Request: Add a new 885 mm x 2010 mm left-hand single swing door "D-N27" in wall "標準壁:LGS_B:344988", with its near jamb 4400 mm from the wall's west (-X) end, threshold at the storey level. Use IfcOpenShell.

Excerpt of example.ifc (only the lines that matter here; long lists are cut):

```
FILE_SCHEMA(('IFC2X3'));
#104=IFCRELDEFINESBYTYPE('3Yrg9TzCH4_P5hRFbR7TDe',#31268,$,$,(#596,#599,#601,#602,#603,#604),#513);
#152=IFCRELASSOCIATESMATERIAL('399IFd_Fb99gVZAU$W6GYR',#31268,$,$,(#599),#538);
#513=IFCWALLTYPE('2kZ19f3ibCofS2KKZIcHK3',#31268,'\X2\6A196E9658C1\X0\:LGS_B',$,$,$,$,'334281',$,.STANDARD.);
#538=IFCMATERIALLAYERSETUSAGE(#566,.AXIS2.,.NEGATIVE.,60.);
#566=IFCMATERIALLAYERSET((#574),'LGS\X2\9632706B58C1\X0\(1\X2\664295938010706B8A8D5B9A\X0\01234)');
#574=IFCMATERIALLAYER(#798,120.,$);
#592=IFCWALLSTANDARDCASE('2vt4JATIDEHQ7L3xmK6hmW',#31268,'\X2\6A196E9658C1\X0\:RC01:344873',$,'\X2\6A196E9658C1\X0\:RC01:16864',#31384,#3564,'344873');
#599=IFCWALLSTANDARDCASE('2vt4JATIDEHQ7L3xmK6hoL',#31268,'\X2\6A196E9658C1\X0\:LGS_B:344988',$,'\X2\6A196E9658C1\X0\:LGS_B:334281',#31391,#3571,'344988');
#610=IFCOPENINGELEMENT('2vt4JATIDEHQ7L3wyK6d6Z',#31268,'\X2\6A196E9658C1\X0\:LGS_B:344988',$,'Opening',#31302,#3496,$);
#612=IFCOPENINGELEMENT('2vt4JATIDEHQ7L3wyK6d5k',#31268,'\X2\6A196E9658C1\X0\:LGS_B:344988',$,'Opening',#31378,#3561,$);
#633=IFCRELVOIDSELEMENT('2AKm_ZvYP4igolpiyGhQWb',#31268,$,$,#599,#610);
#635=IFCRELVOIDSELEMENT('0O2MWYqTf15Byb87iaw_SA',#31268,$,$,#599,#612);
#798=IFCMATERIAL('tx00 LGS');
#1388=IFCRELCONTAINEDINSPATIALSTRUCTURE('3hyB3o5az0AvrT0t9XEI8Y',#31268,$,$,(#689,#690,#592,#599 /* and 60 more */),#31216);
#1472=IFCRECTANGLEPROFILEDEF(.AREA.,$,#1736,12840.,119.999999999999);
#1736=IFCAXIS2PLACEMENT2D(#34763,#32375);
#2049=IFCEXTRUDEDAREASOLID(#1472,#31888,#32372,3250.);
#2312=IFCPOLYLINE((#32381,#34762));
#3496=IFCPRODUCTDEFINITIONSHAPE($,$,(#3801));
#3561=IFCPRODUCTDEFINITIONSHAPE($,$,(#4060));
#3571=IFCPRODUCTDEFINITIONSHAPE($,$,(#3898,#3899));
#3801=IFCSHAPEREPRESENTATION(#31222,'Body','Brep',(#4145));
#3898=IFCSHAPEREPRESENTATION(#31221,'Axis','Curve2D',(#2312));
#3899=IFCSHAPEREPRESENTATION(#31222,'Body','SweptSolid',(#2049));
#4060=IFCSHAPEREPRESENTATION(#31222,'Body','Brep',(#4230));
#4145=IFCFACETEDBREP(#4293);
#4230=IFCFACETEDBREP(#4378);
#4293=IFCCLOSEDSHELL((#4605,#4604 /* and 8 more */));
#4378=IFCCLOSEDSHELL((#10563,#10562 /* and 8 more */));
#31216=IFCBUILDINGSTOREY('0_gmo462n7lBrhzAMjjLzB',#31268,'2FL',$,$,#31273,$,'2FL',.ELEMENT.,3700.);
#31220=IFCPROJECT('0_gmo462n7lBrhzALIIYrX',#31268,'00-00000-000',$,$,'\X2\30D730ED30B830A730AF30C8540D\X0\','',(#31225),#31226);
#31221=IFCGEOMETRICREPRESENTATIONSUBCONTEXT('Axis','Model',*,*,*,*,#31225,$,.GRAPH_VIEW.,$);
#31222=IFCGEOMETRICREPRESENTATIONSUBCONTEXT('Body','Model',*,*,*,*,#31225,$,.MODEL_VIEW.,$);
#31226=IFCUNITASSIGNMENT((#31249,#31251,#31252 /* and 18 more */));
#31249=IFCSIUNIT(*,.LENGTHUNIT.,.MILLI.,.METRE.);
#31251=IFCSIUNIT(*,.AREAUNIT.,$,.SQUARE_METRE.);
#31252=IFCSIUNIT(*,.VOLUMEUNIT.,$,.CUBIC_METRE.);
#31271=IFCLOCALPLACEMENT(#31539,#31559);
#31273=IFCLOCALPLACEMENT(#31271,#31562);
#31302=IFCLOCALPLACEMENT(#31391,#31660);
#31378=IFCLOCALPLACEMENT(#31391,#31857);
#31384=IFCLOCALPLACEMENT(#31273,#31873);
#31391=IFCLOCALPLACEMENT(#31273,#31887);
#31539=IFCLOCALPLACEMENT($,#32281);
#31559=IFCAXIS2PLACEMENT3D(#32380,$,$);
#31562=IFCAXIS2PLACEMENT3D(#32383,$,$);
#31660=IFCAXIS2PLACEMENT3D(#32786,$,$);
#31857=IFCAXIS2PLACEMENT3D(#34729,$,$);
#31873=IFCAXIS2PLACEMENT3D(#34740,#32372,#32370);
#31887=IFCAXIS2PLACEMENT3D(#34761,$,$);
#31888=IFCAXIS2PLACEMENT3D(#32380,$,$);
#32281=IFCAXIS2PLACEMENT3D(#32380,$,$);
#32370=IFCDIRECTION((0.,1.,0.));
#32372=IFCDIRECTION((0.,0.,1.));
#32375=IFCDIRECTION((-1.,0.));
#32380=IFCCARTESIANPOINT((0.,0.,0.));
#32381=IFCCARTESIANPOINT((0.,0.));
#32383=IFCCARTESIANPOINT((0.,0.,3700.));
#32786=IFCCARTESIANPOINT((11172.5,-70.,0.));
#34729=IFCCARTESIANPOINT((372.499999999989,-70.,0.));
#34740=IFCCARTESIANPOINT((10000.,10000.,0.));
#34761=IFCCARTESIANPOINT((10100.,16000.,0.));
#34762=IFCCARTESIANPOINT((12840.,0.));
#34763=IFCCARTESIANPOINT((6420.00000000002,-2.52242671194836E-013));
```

```python
import numpy as np
import ifcopenshell
import ifcopenshell.api.feature
import ifcopenshell.api.geometry
import ifcopenshell.api.root
import ifcopenshell.api.spatial
import ifcopenshell.api.type
import ifcopenshell.geom
import ifcopenshell.util.element
import ifcopenshell.util.placement
import ifcopenshell.util.representation
import ifcopenshell.util.shape
import ifcopenshell.util.unit

model = ifcopenshell.open("example.ifc")
unit_scale = ifcopenshell.util.unit.calculate_unit_scale(model)
settings = ifcopenshell.geom.settings()


def volume(element):
    """Net volume in cubic metres, openings subtracted."""
    shape = ifcopenshell.geom.create_shape(settings, element)
    return ifcopenshell.util.shape.get_volume(shape.geometry)


wall = model.by_guid("2vt4JATIDEHQ7L3xmK6hoL")
storey = ifcopenshell.util.element.get_container(wall, ifc_class="IfcBuildingStorey")
context = ifcopenshell.util.representation.get_context(model, "Model", "Body", "MODEL_VIEW")
before = volume(wall)

width, height, from_end, sill = 0.885, 2.01, 4.4, 0.0  # metres

# The wall runs along its own X axis, and the end named is its -X end.
wall_shape = ifcopenshell.geom.create_shape(settings, wall)
x, y, z = ifcopenshell.util.shape.get_vertices(wall_shape.geometry).T
start = x.min() + from_end
face, thickness = float(y.min()), float(y.max() - y.min())
wall_matrix = ifcopenshell.util.placement.get_local_placement(wall.ObjectPlacement)
level = ifcopenshell.util.placement.get_local_placement(storey.ObjectPlacement)[2, 3]


def in_wall(x, y):
    """Placement at x, y metres in the wall's axes, at sill height."""
    matrix = wall_matrix.copy()
    matrix[:, 3] = wall_matrix @ np.array([x / unit_scale, y / unit_scale, 0.0, 1.0])
    matrix[2, 3] = level + sill / unit_scale
    return matrix


# Opening: a box that overshoots both wall faces by 50 mm.
opening = ifcopenshell.api.root.create_entity(model, ifc_class="IfcOpeningElement")
box = ifcopenshell.api.geometry.add_wall_representation(
    model, context=context, length=width, height=height, thickness=thickness + 0.1
)
ifcopenshell.api.geometry.assign_representation(model, product=opening, representation=box)
ifcopenshell.api.geometry.edit_object_placement(model, product=opening, matrix=in_wall(start, face - 0.05), is_si=False)
ifcopenshell.api.feature.add_feature(model, feature=opening, element=wall)

door = ifcopenshell.api.root.create_entity(model, ifc_class="IfcDoor", name="D-N27")
door.OverallWidth, door.OverallHeight = width / unit_scale, height / unit_scale
body = ifcopenshell.api.geometry.add_door_representation(
    model,
    context=context,
    overall_width=door.OverallWidth,
    overall_height=door.OverallHeight,
    operation_type="SINGLE_SWING_LEFT",
    lining_properties={"LiningDepth": thickness / unit_scale, "ThresholdDepth": thickness / unit_scale},
)
ifcopenshell.api.geometry.assign_representation(model, product=door, representation=body)
ifcopenshell.api.spatial.assign_container(model, products=[door], relating_structure=storey)
fills = ifcopenshell.api.feature.add_filling(model, opening=opening, element=door)
fills.OwnerHistory = door.OwnerHistory  # required in IFC2X3

# IFC2X3 keeps the operation on the door style.
style = ifcopenshell.api.root.create_entity(model, ifc_class="IfcDoorStyle", name="D-N27")
style.OperationType, style.ConstructionType = "SINGLE_SWING_LEFT", "NOTDEFINED"
style.ParameterTakesPrecedence = style.Sizeable = False
ifcopenshell.api.type.assign_type(model, related_objects=[door], relating_type=style)

# The lining spans the wall, so the door starts at the wall face.
ifcopenshell.api.geometry.edit_object_placement(model, product=door, matrix=in_wall(start, face), is_si=False)

after = volume(wall)

print(f"wall volume {before:.3f} -> {after:.3f} m3")

model.write("example-out.ifc")
```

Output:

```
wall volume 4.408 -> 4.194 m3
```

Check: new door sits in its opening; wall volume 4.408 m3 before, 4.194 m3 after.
